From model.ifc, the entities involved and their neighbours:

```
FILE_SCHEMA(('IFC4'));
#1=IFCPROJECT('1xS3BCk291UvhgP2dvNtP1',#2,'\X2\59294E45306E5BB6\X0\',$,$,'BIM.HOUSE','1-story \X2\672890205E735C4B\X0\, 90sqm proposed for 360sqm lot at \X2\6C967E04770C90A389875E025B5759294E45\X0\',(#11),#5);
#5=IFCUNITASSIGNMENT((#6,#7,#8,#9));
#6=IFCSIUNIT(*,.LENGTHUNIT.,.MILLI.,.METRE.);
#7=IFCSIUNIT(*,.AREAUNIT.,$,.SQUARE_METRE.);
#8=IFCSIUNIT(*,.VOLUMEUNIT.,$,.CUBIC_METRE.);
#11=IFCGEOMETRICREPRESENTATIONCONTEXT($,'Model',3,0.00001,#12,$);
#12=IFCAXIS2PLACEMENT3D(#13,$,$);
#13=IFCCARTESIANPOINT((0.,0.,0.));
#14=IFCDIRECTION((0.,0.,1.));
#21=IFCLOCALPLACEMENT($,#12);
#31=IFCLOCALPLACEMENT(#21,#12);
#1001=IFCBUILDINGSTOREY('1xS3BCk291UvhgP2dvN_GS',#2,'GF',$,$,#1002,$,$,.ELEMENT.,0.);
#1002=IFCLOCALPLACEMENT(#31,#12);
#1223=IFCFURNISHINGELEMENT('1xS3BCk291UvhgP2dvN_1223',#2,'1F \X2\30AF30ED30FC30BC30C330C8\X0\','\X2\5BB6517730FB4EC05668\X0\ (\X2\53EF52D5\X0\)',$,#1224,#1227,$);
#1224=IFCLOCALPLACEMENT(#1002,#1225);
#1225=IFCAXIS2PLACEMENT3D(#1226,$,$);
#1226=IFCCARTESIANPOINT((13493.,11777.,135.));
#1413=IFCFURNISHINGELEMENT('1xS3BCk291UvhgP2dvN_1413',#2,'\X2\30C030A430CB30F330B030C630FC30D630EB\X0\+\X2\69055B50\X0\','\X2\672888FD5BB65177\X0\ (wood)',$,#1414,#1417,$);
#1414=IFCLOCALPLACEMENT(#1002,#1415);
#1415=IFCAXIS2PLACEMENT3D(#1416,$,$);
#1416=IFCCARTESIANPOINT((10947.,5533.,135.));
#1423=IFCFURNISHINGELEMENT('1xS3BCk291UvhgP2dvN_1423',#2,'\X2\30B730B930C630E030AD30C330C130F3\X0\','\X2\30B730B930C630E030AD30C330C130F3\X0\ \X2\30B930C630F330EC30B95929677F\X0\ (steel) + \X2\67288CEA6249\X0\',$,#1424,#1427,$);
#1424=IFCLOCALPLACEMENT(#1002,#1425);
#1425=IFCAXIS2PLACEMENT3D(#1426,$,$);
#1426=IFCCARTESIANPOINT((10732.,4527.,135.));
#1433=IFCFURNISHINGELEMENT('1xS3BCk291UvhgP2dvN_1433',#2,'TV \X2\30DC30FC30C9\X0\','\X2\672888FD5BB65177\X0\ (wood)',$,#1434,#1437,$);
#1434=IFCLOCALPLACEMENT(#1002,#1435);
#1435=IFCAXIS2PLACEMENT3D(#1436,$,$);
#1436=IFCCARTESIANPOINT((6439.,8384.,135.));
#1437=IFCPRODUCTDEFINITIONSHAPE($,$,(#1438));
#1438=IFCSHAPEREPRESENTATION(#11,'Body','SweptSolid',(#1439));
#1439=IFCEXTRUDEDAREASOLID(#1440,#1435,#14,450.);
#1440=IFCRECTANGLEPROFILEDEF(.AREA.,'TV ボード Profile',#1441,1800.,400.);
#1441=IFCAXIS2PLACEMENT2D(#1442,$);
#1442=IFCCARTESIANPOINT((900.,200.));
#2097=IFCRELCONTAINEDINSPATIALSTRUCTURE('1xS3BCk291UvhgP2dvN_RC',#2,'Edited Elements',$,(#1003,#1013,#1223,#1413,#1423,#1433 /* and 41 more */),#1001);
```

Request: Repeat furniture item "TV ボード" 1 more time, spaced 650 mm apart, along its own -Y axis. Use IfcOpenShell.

```python
import ifcopenshell
import ifcopenshell.api.geometry
import ifcopenshell.api.root
import ifcopenshell.util.element
import ifcopenshell.util.placement
import ifcopenshell.util.unit

model = ifcopenshell.open("model.ifc")
unit_scale = ifcopenshell.util.unit.calculate_unit_scale(model)


def reuse_history(source, copy):
    """copy_class also copies each property set's owner history, people and application; keep the originals."""
    for rel in copy.IsDefinedBy:
        if rel.is_a("IfcRelDefinesByProperties") and (history := rel.RelatingPropertyDefinition.OwnerHistory):
            rel.RelatingPropertyDefinition.OwnerHistory = source.OwnerHistory
            ifcopenshell.util.element.remove_deep2(model, history)


source = model.by_id(1433)
base = ifcopenshell.util.placement.get_local_placement(source.ObjectPlacement)
step = -base[:3, 1] * 0.65 / unit_scale

for i in range(1, 2):
    copy = ifcopenshell.api.root.copy_class(model, product=source)
    copy.Representation = ifcopenshell.util.element.copy_deep(
        model, source.Representation, exclude=["IfcGeometricRepresentationContext", "IfcRepresentationMap"]
    )
    reuse_history(source, copy)
    matrix = base.copy()
    matrix[:3, 3] += i * step
    print("added at", matrix[:3, 3].round(3) + 0.0)
    ifcopenshell.api.geometry.edit_object_placement(model, product=copy, matrix=matrix, is_si=False)

model.write("model_edited.ifc")
```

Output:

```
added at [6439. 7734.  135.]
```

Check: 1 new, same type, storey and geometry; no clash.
